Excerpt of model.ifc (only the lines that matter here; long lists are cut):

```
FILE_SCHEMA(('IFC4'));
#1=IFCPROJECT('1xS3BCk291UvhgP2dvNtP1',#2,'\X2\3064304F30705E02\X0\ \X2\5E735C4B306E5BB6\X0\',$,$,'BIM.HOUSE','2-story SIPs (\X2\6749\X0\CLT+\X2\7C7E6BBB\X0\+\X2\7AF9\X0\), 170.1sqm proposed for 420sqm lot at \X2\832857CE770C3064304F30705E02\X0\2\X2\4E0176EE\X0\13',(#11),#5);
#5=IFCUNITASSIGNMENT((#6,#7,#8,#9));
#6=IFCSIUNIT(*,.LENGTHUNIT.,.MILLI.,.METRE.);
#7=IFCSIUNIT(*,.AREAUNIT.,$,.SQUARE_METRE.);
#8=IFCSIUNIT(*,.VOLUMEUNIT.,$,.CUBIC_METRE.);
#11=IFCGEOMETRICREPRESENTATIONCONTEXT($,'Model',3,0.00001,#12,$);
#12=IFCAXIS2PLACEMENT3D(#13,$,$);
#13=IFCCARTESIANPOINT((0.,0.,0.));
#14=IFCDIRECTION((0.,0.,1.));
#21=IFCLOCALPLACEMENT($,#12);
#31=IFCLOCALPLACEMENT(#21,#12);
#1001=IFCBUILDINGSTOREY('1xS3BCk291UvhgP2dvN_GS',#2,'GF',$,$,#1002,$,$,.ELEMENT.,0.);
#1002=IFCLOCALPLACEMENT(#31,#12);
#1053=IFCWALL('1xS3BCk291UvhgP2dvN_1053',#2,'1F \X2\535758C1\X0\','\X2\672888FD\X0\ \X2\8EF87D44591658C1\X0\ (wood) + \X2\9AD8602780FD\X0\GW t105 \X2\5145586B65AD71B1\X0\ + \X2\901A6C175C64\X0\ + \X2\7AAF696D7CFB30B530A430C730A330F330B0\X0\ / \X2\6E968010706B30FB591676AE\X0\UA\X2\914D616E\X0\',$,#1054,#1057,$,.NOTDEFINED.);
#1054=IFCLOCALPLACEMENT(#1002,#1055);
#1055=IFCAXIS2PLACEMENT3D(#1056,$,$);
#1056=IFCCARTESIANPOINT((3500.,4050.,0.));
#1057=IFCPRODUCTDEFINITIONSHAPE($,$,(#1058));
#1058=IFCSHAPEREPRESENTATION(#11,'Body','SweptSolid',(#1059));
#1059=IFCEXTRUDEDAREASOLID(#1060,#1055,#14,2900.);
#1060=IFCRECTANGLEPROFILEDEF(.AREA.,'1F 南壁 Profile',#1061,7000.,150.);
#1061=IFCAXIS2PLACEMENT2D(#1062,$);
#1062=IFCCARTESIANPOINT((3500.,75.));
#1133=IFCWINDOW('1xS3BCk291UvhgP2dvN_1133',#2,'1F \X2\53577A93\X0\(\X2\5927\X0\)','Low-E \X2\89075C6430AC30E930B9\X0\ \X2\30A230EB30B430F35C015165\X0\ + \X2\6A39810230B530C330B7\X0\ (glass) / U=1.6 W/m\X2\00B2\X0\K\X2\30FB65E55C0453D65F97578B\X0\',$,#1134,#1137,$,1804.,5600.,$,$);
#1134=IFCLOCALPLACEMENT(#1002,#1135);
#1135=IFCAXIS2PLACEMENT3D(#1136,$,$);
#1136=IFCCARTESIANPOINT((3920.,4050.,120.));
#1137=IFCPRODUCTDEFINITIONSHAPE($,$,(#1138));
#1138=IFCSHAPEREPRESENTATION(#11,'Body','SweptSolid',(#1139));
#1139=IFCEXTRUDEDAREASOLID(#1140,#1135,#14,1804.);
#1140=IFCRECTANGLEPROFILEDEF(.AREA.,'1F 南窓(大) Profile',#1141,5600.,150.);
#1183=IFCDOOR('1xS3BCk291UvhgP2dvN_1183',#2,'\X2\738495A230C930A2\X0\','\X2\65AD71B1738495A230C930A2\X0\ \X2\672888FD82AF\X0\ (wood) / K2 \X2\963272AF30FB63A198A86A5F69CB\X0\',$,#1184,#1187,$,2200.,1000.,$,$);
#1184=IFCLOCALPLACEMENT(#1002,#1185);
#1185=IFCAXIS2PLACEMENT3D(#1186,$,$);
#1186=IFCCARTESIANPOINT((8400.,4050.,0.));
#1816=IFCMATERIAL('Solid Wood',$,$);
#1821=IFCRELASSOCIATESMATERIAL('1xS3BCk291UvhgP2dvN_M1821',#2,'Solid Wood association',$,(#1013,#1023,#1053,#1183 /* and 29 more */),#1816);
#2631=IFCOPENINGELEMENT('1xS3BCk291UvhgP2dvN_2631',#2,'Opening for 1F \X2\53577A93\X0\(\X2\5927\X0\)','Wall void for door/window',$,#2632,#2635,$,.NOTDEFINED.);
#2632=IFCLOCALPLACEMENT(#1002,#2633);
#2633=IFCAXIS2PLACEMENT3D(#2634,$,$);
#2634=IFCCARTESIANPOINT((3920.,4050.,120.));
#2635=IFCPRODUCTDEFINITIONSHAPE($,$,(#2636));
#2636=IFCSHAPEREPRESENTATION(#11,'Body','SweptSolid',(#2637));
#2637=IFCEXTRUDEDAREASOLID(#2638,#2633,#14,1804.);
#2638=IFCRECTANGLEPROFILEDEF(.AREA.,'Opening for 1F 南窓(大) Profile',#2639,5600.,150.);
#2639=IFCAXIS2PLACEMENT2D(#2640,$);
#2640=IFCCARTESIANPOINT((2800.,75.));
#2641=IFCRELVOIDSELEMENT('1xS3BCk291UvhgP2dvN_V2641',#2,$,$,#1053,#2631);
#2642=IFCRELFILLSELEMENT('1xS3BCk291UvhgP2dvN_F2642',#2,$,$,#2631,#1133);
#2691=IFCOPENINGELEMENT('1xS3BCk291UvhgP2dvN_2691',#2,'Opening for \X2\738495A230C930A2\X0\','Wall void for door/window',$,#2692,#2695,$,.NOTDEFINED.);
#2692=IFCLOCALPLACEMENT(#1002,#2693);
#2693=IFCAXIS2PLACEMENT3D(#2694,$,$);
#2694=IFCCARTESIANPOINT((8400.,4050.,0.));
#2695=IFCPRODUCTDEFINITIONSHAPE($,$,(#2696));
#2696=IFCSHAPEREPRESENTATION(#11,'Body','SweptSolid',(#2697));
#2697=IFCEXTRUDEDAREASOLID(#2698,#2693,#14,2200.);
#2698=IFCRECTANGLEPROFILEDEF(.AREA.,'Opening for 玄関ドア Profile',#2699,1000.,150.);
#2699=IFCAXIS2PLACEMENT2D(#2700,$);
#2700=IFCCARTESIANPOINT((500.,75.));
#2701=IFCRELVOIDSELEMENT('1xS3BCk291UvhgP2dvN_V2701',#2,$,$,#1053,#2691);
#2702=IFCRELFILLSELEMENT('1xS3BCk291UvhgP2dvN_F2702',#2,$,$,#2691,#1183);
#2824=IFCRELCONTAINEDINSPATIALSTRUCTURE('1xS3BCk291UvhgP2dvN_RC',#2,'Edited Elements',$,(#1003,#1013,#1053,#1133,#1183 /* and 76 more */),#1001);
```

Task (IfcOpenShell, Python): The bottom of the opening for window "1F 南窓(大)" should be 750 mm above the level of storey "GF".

```python
import numpy as np
import ifcopenshell
import ifcopenshell.api.geometry
import ifcopenshell.geom
import ifcopenshell.util.element
import ifcopenshell.util.placement
import ifcopenshell.util.shape
import ifcopenshell.util.unit

model = ifcopenshell.open("model.ifc")
unit_scale = ifcopenshell.util.unit.calculate_unit_scale(model)

window = model.by_guid("1xS3BCk291UvhgP2dvN_1133")
opening = window.FillsVoids[0].RelatingOpeningElement
storey = ifcopenshell.util.element.get_container(window, ifc_class="IfcBuildingStorey")
level = ifcopenshell.util.placement.get_local_placement(storey.ObjectPlacement)[2, 3]

# The opening's origin need not be at the sill, so measure its lowest point.
shape = ifcopenshell.geom.create_shape(ifcopenshell.geom.settings(), opening)
bottom = ifcopenshell.util.shape.get_shape_bottom_elevation(shape, shape.geometry) / unit_scale
dz = level + 750.0 - bottom

shift = np.array([0.0, 0.0, dz])
# The window is not placed relative to its opening, so move both.
for product in (opening, window):
    matrix = ifcopenshell.util.placement.get_local_placement(product.ObjectPlacement)
    matrix[:3, 3] += shift
    ifcopenshell.api.geometry.edit_object_placement(model, product=product, matrix=matrix, is_si=False)

print(f"moved by {dz * unit_scale:+.3f} m")

model.write("model_rev.ifc")
```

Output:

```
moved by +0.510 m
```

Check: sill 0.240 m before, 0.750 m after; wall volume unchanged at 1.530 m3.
